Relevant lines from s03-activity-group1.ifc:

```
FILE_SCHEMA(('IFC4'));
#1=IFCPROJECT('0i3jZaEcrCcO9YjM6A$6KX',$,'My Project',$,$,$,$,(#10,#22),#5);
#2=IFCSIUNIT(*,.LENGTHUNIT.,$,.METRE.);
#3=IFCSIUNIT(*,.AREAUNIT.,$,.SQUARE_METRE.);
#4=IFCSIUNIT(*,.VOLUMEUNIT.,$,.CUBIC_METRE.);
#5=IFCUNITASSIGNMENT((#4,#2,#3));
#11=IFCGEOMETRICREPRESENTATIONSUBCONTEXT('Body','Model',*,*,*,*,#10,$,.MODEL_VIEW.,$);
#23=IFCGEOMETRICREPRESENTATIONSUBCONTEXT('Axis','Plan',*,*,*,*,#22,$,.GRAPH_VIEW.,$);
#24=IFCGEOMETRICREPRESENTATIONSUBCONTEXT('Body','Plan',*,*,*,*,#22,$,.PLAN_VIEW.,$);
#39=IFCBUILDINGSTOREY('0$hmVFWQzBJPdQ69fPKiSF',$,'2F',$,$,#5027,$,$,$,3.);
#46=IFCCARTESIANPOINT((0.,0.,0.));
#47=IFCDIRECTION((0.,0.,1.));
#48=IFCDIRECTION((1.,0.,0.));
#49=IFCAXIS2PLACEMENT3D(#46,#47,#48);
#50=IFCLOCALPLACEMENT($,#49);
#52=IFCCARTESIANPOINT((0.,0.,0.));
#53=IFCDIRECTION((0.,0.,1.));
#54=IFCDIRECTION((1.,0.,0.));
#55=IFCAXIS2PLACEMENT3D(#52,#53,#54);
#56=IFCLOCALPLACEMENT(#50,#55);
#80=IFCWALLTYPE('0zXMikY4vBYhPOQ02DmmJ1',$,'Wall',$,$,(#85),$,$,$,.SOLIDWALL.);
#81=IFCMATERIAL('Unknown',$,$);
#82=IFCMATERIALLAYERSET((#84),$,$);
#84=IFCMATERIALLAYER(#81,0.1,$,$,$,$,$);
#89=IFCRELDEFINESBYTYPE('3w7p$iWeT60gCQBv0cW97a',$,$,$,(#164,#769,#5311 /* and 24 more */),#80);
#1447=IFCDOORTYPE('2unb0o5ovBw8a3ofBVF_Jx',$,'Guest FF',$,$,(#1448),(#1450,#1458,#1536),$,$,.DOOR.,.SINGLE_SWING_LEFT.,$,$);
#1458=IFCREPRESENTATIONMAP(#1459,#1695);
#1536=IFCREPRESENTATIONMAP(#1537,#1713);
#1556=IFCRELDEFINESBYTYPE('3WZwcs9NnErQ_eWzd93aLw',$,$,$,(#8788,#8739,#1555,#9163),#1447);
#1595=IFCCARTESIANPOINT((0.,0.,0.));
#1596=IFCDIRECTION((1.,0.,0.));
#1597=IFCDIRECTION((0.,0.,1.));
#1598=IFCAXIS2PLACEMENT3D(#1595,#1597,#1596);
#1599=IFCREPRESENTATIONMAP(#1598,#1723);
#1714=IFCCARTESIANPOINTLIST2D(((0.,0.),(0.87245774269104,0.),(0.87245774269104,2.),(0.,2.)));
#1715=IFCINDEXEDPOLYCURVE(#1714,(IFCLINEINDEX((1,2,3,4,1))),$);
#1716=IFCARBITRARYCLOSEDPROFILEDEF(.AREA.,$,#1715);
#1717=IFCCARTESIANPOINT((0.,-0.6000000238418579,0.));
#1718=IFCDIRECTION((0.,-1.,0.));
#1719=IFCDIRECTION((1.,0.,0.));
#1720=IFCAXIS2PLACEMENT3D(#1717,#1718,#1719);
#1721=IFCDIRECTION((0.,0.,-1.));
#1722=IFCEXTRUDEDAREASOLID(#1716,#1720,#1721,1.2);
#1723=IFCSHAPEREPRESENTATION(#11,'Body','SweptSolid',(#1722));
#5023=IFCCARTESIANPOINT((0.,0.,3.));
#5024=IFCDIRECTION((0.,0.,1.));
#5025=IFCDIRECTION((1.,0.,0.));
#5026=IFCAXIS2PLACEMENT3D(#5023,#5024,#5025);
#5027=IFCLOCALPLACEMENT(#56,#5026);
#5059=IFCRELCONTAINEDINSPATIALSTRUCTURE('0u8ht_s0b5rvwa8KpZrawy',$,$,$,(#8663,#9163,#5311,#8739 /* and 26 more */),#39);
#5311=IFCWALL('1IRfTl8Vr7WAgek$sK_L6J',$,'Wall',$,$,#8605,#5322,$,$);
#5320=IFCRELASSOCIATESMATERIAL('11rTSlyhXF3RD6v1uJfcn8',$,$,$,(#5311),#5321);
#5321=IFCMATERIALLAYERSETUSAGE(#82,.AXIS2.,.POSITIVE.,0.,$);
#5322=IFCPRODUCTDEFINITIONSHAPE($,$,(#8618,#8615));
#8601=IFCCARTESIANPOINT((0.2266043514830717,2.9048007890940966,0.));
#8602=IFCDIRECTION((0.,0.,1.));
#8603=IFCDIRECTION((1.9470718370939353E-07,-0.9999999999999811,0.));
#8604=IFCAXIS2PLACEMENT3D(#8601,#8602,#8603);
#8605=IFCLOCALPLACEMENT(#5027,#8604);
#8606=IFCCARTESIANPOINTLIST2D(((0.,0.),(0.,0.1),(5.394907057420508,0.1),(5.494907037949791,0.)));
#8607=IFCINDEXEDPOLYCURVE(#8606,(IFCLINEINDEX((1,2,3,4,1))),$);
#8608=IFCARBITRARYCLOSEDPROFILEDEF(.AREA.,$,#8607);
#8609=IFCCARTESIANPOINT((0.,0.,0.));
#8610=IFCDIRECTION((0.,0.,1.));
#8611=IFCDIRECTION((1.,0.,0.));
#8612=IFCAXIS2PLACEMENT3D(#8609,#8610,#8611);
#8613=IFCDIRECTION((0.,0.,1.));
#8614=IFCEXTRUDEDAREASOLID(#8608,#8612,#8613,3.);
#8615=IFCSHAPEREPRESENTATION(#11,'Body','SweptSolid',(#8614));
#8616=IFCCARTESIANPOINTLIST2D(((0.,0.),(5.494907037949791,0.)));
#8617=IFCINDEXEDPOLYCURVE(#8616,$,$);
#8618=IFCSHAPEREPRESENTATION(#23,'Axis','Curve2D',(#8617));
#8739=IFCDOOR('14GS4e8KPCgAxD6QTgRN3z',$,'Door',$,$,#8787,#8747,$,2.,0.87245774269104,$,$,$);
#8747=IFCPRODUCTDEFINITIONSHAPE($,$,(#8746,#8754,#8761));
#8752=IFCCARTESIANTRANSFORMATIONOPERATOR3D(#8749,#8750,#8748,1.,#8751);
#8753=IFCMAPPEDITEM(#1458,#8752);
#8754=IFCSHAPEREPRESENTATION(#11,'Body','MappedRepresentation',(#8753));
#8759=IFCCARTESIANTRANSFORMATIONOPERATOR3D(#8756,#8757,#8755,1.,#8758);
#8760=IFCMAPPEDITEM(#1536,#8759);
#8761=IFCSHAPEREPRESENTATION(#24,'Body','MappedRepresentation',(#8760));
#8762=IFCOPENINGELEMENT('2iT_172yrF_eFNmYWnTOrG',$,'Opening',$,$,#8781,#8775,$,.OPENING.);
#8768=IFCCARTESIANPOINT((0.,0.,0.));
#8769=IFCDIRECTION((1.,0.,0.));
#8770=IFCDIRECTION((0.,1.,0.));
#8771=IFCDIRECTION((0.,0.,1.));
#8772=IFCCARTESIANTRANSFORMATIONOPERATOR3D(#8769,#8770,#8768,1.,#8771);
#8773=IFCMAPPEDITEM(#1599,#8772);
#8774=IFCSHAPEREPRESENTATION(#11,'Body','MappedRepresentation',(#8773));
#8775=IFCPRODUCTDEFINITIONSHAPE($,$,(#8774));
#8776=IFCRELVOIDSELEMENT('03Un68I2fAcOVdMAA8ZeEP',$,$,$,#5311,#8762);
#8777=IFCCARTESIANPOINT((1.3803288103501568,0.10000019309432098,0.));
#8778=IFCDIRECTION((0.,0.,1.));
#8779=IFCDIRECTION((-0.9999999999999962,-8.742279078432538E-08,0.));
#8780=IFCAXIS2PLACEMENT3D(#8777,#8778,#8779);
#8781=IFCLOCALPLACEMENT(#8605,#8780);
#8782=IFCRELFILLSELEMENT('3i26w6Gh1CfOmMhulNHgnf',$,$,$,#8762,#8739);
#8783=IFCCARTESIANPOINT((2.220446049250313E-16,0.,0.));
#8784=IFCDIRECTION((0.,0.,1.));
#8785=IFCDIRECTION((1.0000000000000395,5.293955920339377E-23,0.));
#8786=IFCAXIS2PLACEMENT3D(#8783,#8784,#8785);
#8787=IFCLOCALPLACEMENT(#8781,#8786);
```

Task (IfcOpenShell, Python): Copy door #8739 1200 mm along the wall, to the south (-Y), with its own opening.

```python
import ifcopenshell
import ifcopenshell.api.feature
import ifcopenshell.api.geometry
import ifcopenshell.api.root
import ifcopenshell.geom
import ifcopenshell.util.element
import ifcopenshell.util.placement
import ifcopenshell.util.shape

model = ifcopenshell.open("s03-activity-group1.ifc")
settings = ifcopenshell.geom.settings()


def volume(element):
    """Net volume in cubic metres, openings subtracted."""
    shape = ifcopenshell.geom.create_shape(settings, element)
    return ifcopenshell.util.shape.get_volume(shape.geometry)


door = model.by_guid("14GS4e8KPCgAxD6QTgRN3z")
opening = door.FillsVoids[0].RelatingOpeningElement
wall = opening.VoidsElements[0].RelatingBuildingElement
before = volume(wall)
shift = ifcopenshell.util.placement.get_local_placement(wall.ObjectPlacement)[:3, 0] * 1.2

# copy_class copies the void relationship, type, container and properties, but no geometry.
new_opening = ifcopenshell.api.root.copy_class(model, product=opening)
new_opening.Representation = ifcopenshell.util.element.copy_deep(
    model, opening.Representation, exclude=["IfcGeometricRepresentationContext", "IfcRepresentationMap"]
)
new_door = ifcopenshell.api.root.copy_class(model, product=door)
new_door.Representation = ifcopenshell.util.element.copy_deep(
    model, door.Representation, exclude=["IfcGeometricRepresentationContext", "IfcRepresentationMap"]
)
ifcopenshell.api.feature.add_filling(model, opening=new_opening, element=new_door)

for old, new in ((opening, new_opening), (door, new_door)):
    matrix = ifcopenshell.util.placement.get_local_placement(old.ObjectPlacement)
    matrix[:3, 3] += shift
    ifcopenshell.api.geometry.edit_object_placement(model, product=new, matrix=matrix, is_si=False)

after = volume(wall)

print(f"wall volume {before:.3f} -> {after:.3f} m3")

model.write("s03-activity-group1_edited.ifc")
```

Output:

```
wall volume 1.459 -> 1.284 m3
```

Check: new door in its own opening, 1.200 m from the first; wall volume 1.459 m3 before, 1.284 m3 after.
